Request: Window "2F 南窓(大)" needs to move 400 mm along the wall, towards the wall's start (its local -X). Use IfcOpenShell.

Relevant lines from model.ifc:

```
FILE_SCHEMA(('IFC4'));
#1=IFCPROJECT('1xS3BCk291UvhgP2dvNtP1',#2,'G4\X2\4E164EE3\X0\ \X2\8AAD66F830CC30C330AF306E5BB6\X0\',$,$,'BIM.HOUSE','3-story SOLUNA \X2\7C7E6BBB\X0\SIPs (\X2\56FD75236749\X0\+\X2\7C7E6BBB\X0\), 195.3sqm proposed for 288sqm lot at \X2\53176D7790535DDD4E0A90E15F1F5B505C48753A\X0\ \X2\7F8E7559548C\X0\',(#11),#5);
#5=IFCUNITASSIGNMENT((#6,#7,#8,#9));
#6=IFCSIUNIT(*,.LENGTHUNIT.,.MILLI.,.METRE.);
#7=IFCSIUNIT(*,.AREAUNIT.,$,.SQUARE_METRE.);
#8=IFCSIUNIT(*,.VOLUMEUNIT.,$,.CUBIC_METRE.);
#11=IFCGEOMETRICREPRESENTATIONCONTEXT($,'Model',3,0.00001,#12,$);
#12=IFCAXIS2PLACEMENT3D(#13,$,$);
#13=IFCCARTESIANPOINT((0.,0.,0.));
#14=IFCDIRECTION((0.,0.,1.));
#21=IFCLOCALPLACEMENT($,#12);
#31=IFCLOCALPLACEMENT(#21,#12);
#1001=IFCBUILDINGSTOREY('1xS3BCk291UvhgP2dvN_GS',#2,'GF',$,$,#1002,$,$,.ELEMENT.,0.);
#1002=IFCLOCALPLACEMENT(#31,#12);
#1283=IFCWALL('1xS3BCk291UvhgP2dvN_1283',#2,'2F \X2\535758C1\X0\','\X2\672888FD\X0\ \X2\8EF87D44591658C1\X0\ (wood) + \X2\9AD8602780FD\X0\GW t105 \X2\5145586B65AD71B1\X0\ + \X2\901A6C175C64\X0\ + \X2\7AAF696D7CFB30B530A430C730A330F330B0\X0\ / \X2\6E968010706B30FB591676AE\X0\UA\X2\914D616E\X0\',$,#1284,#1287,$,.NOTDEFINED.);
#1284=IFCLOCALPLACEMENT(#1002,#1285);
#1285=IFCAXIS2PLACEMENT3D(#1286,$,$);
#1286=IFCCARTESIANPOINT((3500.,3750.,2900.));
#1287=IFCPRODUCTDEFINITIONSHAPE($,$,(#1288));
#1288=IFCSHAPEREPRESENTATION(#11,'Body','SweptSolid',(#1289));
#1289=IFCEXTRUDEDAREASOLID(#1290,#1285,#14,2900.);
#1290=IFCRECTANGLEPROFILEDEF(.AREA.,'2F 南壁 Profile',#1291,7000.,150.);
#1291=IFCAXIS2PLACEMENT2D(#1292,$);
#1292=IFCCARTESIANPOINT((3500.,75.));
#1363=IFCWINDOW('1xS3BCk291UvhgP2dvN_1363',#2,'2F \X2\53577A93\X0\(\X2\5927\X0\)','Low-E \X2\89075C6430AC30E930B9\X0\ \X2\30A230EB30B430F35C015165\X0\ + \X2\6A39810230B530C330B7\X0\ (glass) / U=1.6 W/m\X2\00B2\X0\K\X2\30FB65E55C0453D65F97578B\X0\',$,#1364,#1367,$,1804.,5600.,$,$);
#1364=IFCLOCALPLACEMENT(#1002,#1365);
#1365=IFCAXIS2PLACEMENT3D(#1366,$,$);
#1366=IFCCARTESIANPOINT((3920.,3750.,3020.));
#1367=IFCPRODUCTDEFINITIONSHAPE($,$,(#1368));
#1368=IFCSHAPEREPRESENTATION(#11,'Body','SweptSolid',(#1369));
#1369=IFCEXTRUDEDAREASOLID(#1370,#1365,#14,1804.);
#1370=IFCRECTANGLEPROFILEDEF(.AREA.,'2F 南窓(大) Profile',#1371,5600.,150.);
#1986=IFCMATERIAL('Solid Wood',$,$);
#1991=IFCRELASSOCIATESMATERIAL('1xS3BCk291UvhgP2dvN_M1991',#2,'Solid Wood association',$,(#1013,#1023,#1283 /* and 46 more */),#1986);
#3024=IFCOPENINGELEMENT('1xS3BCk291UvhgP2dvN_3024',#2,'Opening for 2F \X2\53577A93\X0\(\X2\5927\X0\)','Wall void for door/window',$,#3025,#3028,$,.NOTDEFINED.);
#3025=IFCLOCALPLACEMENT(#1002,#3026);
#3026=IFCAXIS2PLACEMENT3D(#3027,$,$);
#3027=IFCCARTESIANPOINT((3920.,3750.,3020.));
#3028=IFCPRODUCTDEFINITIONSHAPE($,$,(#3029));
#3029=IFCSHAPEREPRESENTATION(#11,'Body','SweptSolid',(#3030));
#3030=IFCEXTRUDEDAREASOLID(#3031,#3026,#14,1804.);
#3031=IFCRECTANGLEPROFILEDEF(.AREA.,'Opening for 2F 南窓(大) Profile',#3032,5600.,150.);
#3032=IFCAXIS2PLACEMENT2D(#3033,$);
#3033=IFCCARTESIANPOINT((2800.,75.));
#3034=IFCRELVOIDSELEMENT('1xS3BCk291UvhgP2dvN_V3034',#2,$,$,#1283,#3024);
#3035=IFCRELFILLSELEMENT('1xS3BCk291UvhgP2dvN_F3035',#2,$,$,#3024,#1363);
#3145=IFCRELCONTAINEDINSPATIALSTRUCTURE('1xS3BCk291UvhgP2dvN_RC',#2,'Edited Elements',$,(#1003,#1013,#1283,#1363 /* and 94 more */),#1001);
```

```python
import ifcopenshell
import ifcopenshell.api.geometry
import ifcopenshell.util.placement
import ifcopenshell.util.unit

model = ifcopenshell.open("model.ifc")
unit_scale = ifcopenshell.util.unit.calculate_unit_scale(model)

window = model.by_guid("1xS3BCk291UvhgP2dvN_1363")
opening = window.FillsVoids[0].RelatingOpeningElement
wall = opening.VoidsElements[0].RelatingBuildingElement

wall_matrix = ifcopenshell.util.placement.get_local_placement(wall.ObjectPlacement)
shift = wall_matrix[:3, 0] * -0.4 / unit_scale
before = ifcopenshell.util.placement.get_local_placement(window.ObjectPlacement)[:3, 3].copy()

# The window is not placed relative to its opening, so move both.
for product in (opening, window):
    matrix = ifcopenshell.util.placement.get_local_placement(product.ObjectPlacement)
    matrix[:3, 3] += shift
    ifcopenshell.api.geometry.edit_object_placement(model, product=product, matrix=matrix, is_si=False)

after = ifcopenshell.util.placement.get_local_placement(window.ObjectPlacement)[:3, 3]
print("window moved by", (after - before).round(3) + 0.0)

model.write("model-out.ifc")
```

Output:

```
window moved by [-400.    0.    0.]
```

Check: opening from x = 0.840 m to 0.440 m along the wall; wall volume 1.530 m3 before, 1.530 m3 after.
